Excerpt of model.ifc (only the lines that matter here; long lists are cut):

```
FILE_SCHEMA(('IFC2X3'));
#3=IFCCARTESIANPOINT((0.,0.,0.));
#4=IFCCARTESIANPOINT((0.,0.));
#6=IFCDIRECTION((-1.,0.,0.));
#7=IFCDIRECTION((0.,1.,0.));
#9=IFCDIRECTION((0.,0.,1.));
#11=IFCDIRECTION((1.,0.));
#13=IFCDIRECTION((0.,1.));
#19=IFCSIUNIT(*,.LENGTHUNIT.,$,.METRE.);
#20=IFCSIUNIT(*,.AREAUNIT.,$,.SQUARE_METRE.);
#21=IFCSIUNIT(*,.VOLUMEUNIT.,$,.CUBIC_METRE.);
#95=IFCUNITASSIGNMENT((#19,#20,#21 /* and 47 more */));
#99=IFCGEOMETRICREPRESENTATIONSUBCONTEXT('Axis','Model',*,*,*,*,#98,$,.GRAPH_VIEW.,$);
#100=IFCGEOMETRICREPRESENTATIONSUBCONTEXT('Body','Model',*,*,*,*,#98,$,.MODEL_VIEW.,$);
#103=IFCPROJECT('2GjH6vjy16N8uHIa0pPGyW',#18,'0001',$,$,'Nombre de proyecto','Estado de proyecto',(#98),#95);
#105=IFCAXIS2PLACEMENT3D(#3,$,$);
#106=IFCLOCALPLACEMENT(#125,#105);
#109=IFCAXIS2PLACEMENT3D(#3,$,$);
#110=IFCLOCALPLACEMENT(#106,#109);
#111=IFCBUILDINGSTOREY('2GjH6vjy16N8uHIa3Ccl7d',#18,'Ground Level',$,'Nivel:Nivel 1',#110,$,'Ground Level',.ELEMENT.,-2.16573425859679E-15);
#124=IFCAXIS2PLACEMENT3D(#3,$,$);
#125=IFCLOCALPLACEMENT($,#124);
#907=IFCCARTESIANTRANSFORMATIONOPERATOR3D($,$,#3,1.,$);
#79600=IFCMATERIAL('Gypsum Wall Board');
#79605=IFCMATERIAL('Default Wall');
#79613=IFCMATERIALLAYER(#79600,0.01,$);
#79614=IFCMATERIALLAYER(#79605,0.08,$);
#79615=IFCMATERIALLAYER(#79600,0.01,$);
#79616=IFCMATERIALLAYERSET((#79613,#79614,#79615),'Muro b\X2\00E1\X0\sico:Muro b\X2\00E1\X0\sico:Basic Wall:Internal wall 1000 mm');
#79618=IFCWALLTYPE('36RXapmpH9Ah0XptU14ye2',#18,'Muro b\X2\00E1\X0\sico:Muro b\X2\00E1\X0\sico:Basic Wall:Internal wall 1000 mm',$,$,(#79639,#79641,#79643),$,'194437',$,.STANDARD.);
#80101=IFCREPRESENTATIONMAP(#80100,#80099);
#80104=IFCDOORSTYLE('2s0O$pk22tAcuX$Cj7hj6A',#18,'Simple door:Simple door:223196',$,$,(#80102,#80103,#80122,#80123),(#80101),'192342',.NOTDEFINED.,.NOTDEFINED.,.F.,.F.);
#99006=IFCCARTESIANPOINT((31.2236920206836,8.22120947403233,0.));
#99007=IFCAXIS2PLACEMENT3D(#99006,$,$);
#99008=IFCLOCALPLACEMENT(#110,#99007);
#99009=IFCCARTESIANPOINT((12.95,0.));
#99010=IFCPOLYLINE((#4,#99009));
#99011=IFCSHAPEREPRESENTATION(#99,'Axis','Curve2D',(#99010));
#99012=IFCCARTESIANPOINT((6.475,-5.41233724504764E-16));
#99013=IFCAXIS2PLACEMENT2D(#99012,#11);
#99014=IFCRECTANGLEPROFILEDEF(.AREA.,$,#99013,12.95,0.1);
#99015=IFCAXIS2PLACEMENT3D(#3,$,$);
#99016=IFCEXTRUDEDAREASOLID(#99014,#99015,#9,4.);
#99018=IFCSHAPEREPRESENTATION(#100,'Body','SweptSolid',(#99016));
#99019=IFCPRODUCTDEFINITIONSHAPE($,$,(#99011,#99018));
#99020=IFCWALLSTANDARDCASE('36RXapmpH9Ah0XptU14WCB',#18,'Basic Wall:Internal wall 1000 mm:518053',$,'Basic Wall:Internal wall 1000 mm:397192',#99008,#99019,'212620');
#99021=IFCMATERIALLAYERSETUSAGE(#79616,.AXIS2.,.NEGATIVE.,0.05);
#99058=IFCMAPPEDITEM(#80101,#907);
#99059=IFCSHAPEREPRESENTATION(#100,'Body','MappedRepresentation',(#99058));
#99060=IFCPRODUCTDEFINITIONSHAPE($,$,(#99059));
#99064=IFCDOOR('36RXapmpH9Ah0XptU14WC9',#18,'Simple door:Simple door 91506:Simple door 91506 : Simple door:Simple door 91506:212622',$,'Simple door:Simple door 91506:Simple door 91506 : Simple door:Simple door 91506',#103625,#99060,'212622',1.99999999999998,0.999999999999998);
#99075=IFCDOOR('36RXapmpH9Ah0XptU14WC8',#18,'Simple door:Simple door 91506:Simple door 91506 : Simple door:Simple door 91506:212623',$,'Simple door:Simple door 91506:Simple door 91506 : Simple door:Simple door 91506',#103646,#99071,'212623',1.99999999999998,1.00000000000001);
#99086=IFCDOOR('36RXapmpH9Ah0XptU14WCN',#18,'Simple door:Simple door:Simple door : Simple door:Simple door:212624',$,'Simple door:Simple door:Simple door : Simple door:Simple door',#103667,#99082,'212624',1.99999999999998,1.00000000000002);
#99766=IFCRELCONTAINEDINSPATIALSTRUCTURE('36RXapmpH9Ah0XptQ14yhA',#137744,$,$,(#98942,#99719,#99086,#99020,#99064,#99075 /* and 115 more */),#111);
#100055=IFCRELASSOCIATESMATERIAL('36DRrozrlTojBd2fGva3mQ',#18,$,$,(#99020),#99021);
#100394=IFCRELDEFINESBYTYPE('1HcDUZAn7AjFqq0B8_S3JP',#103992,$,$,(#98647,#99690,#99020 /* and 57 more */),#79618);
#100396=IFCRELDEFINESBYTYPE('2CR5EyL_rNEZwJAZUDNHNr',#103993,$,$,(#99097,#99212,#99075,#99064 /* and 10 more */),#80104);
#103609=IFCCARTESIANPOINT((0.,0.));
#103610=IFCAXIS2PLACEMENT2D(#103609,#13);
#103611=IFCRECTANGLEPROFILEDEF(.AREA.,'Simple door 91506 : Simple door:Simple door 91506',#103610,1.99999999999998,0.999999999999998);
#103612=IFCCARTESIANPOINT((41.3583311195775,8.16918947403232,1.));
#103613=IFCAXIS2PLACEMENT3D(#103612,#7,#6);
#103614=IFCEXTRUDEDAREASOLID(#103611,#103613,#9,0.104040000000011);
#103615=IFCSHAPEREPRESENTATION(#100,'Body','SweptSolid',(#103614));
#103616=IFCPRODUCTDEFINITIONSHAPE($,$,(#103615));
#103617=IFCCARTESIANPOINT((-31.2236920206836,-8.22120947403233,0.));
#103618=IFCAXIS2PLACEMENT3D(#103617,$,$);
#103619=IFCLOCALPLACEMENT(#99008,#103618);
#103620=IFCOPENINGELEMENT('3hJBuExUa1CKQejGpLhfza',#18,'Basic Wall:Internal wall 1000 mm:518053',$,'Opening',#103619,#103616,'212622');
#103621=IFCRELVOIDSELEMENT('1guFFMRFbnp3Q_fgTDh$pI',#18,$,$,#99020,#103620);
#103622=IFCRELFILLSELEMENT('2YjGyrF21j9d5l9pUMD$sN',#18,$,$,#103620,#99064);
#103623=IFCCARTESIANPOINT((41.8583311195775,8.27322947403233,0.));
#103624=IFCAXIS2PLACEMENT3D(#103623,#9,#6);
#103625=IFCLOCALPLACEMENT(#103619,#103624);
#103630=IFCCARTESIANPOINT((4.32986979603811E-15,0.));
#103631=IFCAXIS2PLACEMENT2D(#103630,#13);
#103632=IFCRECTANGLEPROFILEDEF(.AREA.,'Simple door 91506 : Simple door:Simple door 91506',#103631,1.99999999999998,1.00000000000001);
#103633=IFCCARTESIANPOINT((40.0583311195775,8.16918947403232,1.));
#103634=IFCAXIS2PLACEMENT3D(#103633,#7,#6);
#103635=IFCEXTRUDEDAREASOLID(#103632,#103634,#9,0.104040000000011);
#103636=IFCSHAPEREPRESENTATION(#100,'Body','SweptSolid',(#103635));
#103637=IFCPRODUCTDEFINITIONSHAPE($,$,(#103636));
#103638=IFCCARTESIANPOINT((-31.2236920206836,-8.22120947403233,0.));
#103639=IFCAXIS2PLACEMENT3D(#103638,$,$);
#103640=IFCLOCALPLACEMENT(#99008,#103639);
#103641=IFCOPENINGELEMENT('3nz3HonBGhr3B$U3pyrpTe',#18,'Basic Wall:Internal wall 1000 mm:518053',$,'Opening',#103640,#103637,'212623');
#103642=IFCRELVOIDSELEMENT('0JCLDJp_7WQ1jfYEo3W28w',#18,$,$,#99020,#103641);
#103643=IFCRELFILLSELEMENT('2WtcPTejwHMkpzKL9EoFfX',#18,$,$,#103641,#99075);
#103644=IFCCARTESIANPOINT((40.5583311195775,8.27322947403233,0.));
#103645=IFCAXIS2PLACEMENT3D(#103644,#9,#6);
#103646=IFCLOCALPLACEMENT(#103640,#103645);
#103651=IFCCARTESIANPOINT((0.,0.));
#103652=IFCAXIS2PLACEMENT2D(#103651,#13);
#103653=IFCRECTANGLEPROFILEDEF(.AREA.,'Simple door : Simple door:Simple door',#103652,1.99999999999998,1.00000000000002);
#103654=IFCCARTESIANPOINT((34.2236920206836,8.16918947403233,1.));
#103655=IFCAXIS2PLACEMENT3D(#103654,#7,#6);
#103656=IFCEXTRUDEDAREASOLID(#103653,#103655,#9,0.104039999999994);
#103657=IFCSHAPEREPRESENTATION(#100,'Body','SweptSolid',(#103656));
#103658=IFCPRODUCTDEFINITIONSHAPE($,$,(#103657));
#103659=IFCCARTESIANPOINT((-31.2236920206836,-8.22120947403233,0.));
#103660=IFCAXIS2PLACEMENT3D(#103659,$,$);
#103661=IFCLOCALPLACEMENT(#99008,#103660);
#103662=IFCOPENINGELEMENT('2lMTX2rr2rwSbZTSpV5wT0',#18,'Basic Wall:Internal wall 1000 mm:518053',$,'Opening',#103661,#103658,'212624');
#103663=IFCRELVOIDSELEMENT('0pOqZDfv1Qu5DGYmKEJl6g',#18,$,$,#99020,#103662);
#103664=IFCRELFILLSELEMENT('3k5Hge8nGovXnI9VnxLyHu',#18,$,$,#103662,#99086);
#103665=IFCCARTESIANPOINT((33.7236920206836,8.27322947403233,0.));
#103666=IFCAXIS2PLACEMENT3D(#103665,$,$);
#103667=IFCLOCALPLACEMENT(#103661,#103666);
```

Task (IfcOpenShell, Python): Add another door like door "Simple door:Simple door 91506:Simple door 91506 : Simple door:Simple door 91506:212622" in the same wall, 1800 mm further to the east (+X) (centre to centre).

```python
import ifcopenshell
import ifcopenshell.api.feature
import ifcopenshell.api.geometry
import ifcopenshell.api.root
import ifcopenshell.geom
import ifcopenshell.util.element
import ifcopenshell.util.placement
import ifcopenshell.util.shape
import ifcopenshell.util.unit

model = ifcopenshell.open("model.ifc")
unit_scale = ifcopenshell.util.unit.calculate_unit_scale(model)
settings = ifcopenshell.geom.settings()


def volume(element):
    """Net volume in cubic metres, openings subtracted."""
    shape = ifcopenshell.geom.create_shape(settings, element)
    return ifcopenshell.util.shape.get_volume(shape.geometry)


def reuse_history(source, copy):
    """copy_class also copies each property set's owner history, people and application; keep the originals."""
    for rel in copy.IsDefinedBy:
        if rel.is_a("IfcRelDefinesByProperties") and (history := rel.RelatingPropertyDefinition.OwnerHistory):
            rel.RelatingPropertyDefinition.OwnerHistory = source.OwnerHistory
            ifcopenshell.util.element.remove_deep2(model, history)


door = model.by_guid("36RXapmpH9Ah0XptU14WC9")
opening = door.FillsVoids[0].RelatingOpeningElement
wall = opening.VoidsElements[0].RelatingBuildingElement
before = volume(wall)
shift = ifcopenshell.util.placement.get_local_placement(wall.ObjectPlacement)[:3, 0] * 1.8 / unit_scale

# copy_class copies the void relationship, type, container and properties, but no geometry.
new_opening = ifcopenshell.api.root.copy_class(model, product=opening)
new_opening.Representation = ifcopenshell.util.element.copy_deep(
    model, opening.Representation, exclude=["IfcGeometricRepresentationContext", "IfcRepresentationMap"]
)
new_opening.Name = "Basic Wall:Internal wall 1000 mm"
new_opening.Tag = None
new_door = ifcopenshell.api.root.copy_class(model, product=door)
new_door.Representation = ifcopenshell.util.element.copy_deep(
    model, door.Representation, exclude=["IfcGeometricRepresentationContext", "IfcRepresentationMap"]
)
new_door.Name = "Simple door:Simple door 91506:Simple door 91506 : Simple door:Simple door 91506"
new_door.Tag = None
reuse_history(door, new_door)
fills = ifcopenshell.api.feature.add_filling(model, opening=new_opening, element=new_door)
fills.OwnerHistory = new_door.OwnerHistory  # required in IFC2X3

for old, new in ((opening, new_opening), (door, new_door)):
    matrix = ifcopenshell.util.placement.get_local_placement(old.ObjectPlacement)
    matrix[:3, 3] += shift
    ifcopenshell.api.geometry.edit_object_placement(model, product=new, matrix=matrix, is_si=False)

after = volume(wall)

print(f"wall volume {before:.3f} -> {after:.3f} m3")

model.write("model_rev.ifc")
```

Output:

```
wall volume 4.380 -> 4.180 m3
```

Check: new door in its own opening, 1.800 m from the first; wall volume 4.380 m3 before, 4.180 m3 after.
